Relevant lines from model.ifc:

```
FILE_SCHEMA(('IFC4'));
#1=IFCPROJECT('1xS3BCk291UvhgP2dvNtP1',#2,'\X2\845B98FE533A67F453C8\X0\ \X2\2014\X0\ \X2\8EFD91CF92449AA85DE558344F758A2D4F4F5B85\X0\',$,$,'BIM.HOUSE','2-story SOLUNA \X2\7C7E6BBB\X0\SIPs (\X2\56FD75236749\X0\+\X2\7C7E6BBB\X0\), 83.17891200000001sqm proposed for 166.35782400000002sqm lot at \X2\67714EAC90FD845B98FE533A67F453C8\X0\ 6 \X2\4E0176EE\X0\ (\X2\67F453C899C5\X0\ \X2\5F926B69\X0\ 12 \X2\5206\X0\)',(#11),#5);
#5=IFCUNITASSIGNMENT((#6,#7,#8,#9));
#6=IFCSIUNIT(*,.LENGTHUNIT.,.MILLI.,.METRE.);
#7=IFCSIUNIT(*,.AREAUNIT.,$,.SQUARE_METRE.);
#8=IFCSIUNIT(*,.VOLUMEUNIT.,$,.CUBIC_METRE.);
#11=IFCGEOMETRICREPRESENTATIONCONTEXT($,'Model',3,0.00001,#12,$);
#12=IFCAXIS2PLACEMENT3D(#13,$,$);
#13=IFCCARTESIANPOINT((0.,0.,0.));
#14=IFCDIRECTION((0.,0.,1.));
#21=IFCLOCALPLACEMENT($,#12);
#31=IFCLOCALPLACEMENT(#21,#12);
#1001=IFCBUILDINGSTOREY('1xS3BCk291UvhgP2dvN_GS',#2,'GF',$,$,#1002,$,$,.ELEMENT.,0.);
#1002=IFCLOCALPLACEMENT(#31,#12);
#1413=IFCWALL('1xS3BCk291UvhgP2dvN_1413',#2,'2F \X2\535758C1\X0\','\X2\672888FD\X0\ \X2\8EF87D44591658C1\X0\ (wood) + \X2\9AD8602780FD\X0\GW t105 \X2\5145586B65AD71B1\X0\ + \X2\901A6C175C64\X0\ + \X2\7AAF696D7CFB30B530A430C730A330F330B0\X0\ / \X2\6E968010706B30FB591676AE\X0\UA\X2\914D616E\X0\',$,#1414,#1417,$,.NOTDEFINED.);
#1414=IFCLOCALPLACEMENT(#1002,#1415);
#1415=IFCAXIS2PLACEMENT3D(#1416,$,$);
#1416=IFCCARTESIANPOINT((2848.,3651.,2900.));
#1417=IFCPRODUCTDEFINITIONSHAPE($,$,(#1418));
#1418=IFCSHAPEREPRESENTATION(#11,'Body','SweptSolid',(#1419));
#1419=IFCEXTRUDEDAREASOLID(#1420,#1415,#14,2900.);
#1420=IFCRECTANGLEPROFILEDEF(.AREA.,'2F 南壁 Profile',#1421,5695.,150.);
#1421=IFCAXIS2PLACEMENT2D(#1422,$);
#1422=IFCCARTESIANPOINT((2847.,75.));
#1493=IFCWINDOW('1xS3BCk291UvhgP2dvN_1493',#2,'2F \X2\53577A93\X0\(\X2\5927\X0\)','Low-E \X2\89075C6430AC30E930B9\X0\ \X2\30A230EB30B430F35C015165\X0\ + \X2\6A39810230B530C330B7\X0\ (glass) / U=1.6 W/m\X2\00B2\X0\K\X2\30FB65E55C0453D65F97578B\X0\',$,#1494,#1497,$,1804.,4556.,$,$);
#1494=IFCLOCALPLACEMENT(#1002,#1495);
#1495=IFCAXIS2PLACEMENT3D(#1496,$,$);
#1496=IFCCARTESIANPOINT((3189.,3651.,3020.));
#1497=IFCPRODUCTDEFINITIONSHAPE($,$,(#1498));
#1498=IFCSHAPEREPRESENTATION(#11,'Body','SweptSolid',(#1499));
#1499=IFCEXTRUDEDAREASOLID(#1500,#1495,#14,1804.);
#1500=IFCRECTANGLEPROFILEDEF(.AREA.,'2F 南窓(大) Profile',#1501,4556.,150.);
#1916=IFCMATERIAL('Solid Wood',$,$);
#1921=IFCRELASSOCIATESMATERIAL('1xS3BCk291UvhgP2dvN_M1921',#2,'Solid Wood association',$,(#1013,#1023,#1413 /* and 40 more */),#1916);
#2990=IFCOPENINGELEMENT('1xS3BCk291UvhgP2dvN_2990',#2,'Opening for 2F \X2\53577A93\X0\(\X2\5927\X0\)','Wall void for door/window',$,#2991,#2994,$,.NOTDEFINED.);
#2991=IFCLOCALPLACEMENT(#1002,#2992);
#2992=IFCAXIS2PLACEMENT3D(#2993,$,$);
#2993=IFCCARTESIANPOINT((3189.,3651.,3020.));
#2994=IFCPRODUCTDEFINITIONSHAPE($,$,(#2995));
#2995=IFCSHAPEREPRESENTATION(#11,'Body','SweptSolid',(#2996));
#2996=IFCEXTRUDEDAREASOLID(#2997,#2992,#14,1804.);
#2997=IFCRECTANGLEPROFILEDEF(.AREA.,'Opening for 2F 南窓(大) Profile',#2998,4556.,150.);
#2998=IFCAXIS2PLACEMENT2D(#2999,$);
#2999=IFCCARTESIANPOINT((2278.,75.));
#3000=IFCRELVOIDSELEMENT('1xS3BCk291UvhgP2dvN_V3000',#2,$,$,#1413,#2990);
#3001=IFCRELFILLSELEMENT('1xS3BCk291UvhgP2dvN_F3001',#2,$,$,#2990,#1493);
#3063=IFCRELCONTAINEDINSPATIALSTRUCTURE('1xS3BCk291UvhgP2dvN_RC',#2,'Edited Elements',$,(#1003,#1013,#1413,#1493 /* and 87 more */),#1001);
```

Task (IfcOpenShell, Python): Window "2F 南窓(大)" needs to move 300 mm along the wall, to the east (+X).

```python
import ifcopenshell
import ifcopenshell.api.geometry
import ifcopenshell.util.placement

model = ifcopenshell.open("model.ifc")

window = model.by_guid("1xS3BCk291UvhgP2dvN_1493")
opening = window.FillsVoids[0].RelatingOpeningElement
wall = opening.VoidsElements[0].RelatingBuildingElement

wall_matrix = ifcopenshell.util.placement.get_local_placement(wall.ObjectPlacement)
shift = wall_matrix[:3, 0] * 300.0
before = ifcopenshell.util.placement.get_local_placement(window.ObjectPlacement)[:3, 3].copy()

# The window is not placed relative to its opening, so move both.
for product in (opening, window):
    matrix = ifcopenshell.util.placement.get_local_placement(product.ObjectPlacement)
    matrix[:3, 3] += shift
    ifcopenshell.api.geometry.edit_object_placement(model, product=product, matrix=matrix, is_si=False)

after = ifcopenshell.util.placement.get_local_placement(window.ObjectPlacement)[:3, 3]
print("window moved by", (after - before).round(3) + 0.0)

model.write("model_rev.ifc")
```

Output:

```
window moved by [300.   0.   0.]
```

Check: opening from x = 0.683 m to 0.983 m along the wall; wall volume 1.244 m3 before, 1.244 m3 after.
